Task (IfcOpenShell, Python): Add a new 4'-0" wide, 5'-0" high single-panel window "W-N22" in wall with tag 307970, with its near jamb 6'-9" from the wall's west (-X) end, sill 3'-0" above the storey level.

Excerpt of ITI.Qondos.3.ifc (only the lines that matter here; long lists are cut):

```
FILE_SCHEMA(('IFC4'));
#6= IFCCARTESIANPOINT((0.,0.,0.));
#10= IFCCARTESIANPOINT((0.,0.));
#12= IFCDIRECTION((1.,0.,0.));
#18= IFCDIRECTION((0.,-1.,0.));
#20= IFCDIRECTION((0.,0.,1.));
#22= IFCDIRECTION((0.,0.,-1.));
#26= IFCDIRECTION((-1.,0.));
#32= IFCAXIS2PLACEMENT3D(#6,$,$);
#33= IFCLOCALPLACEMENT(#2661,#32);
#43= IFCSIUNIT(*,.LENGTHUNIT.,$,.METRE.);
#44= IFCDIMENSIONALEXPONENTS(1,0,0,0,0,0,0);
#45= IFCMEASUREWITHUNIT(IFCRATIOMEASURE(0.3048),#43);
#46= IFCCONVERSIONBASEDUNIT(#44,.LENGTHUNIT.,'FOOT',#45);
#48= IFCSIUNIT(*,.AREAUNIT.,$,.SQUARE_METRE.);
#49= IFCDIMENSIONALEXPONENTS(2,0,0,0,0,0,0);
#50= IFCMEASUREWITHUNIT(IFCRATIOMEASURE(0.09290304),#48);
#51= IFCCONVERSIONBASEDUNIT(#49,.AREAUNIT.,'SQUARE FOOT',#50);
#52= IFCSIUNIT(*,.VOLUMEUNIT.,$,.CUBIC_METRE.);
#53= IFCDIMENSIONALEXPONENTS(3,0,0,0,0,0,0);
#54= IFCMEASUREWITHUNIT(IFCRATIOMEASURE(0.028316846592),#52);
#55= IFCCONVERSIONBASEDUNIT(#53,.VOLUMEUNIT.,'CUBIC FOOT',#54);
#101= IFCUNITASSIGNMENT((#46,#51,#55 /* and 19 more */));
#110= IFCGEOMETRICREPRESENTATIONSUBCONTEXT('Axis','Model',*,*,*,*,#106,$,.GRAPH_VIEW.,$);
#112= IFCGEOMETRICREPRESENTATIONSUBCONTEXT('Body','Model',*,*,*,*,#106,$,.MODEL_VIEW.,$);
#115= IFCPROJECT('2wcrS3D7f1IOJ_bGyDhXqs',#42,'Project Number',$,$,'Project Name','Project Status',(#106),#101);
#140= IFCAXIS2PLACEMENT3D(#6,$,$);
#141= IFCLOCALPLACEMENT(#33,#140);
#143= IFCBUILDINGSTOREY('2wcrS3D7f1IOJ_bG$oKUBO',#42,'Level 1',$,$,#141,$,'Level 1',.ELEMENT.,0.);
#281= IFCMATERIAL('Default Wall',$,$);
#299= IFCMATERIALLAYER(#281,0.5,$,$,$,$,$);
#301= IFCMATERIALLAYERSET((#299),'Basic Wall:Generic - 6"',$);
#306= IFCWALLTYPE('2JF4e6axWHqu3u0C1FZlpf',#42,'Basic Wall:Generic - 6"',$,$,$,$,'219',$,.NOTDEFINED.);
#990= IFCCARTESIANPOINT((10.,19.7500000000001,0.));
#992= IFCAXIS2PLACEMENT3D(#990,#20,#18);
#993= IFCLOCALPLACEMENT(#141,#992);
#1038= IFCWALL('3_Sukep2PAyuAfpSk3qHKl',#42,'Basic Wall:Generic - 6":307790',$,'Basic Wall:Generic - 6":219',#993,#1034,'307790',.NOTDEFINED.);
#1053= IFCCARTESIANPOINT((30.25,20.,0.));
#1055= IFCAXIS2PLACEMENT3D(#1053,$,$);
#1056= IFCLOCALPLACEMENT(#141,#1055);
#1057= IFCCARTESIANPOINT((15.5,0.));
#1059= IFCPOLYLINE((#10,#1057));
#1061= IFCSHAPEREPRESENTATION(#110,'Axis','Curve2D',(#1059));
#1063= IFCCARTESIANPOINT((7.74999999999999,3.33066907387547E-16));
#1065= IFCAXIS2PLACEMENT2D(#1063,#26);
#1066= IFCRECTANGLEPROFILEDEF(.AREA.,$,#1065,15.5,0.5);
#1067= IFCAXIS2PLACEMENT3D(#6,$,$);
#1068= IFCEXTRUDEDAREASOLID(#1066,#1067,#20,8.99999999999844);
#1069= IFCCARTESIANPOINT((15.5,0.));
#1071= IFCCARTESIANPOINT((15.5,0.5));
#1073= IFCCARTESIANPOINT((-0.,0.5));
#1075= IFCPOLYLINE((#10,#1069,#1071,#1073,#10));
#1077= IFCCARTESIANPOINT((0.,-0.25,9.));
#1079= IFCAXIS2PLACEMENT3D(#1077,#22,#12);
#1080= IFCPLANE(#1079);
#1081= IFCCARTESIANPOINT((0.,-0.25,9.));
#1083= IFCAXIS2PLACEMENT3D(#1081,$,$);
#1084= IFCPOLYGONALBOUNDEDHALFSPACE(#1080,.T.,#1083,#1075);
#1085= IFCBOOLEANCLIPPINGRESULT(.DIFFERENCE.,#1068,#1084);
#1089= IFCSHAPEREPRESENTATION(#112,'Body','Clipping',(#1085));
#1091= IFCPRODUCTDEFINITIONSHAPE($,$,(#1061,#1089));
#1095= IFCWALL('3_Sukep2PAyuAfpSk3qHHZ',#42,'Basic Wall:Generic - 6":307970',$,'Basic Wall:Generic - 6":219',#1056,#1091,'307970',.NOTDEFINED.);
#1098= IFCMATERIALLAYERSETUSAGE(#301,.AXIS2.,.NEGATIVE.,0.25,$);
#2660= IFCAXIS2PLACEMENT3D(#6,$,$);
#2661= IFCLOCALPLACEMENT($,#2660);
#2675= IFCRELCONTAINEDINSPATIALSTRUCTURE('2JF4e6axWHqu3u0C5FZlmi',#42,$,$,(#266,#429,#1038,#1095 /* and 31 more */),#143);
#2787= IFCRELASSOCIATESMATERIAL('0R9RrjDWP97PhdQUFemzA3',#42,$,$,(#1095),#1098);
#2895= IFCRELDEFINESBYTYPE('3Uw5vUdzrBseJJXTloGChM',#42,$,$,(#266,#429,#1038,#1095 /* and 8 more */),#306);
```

```python
import numpy as np
import ifcopenshell
import ifcopenshell.api.feature
import ifcopenshell.api.geometry
import ifcopenshell.api.root
import ifcopenshell.api.spatial
import ifcopenshell.geom
import ifcopenshell.util.element
import ifcopenshell.util.placement
import ifcopenshell.util.representation
import ifcopenshell.util.shape
import ifcopenshell.util.unit

model = ifcopenshell.open("ITI.Qondos.3.ifc")
unit_scale = ifcopenshell.util.unit.calculate_unit_scale(model)
settings = ifcopenshell.geom.settings()


def volume(element):
    """Net volume in cubic metres, openings subtracted."""
    shape = ifcopenshell.geom.create_shape(settings, element)
    return ifcopenshell.util.shape.get_volume(shape.geometry)


wall = model.by_guid("3_Sukep2PAyuAfpSk3qHHZ")
storey = ifcopenshell.util.element.get_container(wall, ifc_class="IfcBuildingStorey")
context = ifcopenshell.util.representation.get_context(model, "Model", "Body", "MODEL_VIEW")
before = volume(wall)

width, height, from_end, sill = 1.2192, 1.524, 2.0574, 0.9144  # metres

# The wall runs along its own X axis, and the end named is its -X end.
wall_shape = ifcopenshell.geom.create_shape(settings, wall)
x, y, z = ifcopenshell.util.shape.get_vertices(wall_shape.geometry).T
start = x.min() + from_end
face, thickness = float(y.min()), float(y.max() - y.min())
wall_matrix = ifcopenshell.util.placement.get_local_placement(wall.ObjectPlacement)
level = ifcopenshell.util.placement.get_local_placement(storey.ObjectPlacement)[2, 3]


def in_wall(x, y):
    """Placement at x, y metres in the wall's axes, at sill height."""
    matrix = wall_matrix.copy()
    matrix[:, 3] = wall_matrix @ np.array([x / unit_scale, y / unit_scale, 0.0, 1.0])
    matrix[2, 3] = level + sill / unit_scale
    return matrix


# Opening: a box that overshoots both wall faces by 50 mm.
opening = ifcopenshell.api.root.create_entity(model, ifc_class="IfcOpeningElement", predefined_type="OPENING")
box = ifcopenshell.api.geometry.add_wall_representation(
    model, context=context, length=width, height=height, thickness=thickness + 0.1
)
ifcopenshell.api.geometry.assign_representation(model, product=opening, representation=box)
ifcopenshell.api.geometry.edit_object_placement(model, product=opening, matrix=in_wall(start, face - 0.05), is_si=False)
ifcopenshell.api.feature.add_feature(model, feature=opening, element=wall)

window = ifcopenshell.api.root.create_entity(model, ifc_class="IfcWindow", name="W-N22", predefined_type="WINDOW")
window.OverallWidth, window.OverallHeight = width / unit_scale, height / unit_scale
window.PartitioningType = "SINGLE_PANEL"
body = ifcopenshell.api.geometry.add_window_representation(
    model,
    context=context,
    overall_width=window.OverallWidth,
    overall_height=window.OverallHeight,
    partition_type="SINGLE_PANEL",
)
ifcopenshell.api.geometry.assign_representation(model, product=window, representation=body)
ifcopenshell.api.spatial.assign_container(model, products=[window], relating_structure=storey)
ifcopenshell.api.feature.add_filling(model, opening=opening, element=window)

# Centre the window in the wall's thickness.
ifcopenshell.api.geometry.edit_object_placement(model, product=window, matrix=in_wall(start, face), is_si=False)
window_shape = ifcopenshell.geom.create_shape(settings, window)
depth = ifcopenshell.util.shape.get_vertices(window_shape.geometry)[:, 1]
offset = face + thickness / 2 - (depth.min() + depth.max()) / 2
ifcopenshell.api.geometry.edit_object_placement(model, product=window, matrix=in_wall(start, offset), is_si=False)

after = volume(wall)

print(f"wall volume {before:.3f} -> {after:.3f} m3")

model.write("ITI.Qondos.3_v2.ifc")
```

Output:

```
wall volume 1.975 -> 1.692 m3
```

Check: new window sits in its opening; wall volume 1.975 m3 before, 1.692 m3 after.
